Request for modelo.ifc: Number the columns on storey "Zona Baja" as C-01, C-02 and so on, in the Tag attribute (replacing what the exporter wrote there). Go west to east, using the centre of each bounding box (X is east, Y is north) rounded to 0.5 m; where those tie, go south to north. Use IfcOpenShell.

First a look at what the model holds.

```python
import ifcopenshell
import ifcopenshell.util.element
import ifcopenshell.util.placement

model = ifcopenshell.open("modelo.ifc")
print(model.schema)
storey = next(s for s in model.by_type("IfcBuildingStorey") if s.Name == "Zona Baja")
columns = [e for e in ifcopenshell.util.element.get_decomposition(storey) if e.is_a("IfcColumn")]
for e in sorted(columns, key=lambda e: e.id()):
    origin = ifcopenshell.util.placement.get_local_placement(e.ObjectPlacement)[:3, 3]
    print(e.id(), e.Tag, e.Name, origin.round(2) + 0.0, sep=" | ")
```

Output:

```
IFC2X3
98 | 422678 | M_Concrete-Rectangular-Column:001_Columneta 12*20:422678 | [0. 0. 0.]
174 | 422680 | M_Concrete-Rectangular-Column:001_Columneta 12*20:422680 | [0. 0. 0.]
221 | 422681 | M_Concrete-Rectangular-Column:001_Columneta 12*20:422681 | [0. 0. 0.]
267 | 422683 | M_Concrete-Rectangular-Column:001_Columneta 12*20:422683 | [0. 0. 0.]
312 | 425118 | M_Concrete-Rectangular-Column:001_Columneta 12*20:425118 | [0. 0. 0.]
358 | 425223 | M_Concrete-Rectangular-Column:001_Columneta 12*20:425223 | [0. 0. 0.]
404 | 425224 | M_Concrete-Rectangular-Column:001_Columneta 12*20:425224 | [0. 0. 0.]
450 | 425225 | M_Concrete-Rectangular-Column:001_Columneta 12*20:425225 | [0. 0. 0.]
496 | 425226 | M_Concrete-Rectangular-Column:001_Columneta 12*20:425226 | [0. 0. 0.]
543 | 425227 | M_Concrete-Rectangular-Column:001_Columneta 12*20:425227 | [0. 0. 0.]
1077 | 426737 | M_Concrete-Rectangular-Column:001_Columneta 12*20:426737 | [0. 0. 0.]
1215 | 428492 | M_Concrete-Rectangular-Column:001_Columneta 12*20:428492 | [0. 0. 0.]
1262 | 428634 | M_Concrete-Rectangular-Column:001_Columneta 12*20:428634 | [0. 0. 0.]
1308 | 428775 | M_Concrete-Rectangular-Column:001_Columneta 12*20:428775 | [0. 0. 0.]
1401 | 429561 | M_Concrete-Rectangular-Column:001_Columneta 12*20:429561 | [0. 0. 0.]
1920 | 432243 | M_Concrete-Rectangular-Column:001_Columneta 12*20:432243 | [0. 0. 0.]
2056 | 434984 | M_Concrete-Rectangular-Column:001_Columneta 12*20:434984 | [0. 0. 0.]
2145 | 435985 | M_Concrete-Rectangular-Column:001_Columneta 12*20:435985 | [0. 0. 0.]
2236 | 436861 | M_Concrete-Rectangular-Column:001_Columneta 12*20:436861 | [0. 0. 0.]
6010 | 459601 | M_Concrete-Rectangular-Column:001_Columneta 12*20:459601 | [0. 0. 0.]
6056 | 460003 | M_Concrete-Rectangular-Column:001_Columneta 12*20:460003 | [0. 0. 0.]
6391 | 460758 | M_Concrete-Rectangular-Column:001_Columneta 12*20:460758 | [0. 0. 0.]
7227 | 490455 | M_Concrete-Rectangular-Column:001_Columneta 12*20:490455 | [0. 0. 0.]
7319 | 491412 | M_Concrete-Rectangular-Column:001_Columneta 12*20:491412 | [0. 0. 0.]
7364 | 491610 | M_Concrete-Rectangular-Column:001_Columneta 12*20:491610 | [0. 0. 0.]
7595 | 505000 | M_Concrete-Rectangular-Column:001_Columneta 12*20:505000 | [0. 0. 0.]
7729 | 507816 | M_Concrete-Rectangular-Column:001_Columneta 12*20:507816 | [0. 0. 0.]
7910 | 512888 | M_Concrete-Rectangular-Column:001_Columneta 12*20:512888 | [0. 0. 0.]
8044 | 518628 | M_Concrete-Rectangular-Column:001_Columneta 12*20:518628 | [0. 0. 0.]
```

```python
import ifcopenshell
import ifcopenshell.geom
import ifcopenshell.util.element
import ifcopenshell.util.shape

model = ifcopenshell.open("modelo.ifc")
settings = ifcopenshell.geom.settings()
settings.set("use-world-coords", True)


def centre(element):
    shape = ifcopenshell.geom.create_shape(settings, element)
    return ifcopenshell.util.shape.get_bbox_centroid(shape.geometry)


storey = next(s for s in model.by_type("IfcBuildingStorey") if s.Name == "Zona Baja")
columns = [e for e in ifcopenshell.util.element.get_decomposition(storey) if e.is_a("IfcColumn")]

# Insertion points can sit at a corner or the storey origin, so sort by the geometry (in metres).
centres = {e: centre(e) for e in columns}
columns.sort(key=lambda e: (round(centres[e][0] / 0.5), centres[e][1]))

for i, e in enumerate(columns, start=1):
    number = f"C-{i:02d}"
    e.Tag = number
    print(e.id(), number)

model.write("modelo-out.ifc")
```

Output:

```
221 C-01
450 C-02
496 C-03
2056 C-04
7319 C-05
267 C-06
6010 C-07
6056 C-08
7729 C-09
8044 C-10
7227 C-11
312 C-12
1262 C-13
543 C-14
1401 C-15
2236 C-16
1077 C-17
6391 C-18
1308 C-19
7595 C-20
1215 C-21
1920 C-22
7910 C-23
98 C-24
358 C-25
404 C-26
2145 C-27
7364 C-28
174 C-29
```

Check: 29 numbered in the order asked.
